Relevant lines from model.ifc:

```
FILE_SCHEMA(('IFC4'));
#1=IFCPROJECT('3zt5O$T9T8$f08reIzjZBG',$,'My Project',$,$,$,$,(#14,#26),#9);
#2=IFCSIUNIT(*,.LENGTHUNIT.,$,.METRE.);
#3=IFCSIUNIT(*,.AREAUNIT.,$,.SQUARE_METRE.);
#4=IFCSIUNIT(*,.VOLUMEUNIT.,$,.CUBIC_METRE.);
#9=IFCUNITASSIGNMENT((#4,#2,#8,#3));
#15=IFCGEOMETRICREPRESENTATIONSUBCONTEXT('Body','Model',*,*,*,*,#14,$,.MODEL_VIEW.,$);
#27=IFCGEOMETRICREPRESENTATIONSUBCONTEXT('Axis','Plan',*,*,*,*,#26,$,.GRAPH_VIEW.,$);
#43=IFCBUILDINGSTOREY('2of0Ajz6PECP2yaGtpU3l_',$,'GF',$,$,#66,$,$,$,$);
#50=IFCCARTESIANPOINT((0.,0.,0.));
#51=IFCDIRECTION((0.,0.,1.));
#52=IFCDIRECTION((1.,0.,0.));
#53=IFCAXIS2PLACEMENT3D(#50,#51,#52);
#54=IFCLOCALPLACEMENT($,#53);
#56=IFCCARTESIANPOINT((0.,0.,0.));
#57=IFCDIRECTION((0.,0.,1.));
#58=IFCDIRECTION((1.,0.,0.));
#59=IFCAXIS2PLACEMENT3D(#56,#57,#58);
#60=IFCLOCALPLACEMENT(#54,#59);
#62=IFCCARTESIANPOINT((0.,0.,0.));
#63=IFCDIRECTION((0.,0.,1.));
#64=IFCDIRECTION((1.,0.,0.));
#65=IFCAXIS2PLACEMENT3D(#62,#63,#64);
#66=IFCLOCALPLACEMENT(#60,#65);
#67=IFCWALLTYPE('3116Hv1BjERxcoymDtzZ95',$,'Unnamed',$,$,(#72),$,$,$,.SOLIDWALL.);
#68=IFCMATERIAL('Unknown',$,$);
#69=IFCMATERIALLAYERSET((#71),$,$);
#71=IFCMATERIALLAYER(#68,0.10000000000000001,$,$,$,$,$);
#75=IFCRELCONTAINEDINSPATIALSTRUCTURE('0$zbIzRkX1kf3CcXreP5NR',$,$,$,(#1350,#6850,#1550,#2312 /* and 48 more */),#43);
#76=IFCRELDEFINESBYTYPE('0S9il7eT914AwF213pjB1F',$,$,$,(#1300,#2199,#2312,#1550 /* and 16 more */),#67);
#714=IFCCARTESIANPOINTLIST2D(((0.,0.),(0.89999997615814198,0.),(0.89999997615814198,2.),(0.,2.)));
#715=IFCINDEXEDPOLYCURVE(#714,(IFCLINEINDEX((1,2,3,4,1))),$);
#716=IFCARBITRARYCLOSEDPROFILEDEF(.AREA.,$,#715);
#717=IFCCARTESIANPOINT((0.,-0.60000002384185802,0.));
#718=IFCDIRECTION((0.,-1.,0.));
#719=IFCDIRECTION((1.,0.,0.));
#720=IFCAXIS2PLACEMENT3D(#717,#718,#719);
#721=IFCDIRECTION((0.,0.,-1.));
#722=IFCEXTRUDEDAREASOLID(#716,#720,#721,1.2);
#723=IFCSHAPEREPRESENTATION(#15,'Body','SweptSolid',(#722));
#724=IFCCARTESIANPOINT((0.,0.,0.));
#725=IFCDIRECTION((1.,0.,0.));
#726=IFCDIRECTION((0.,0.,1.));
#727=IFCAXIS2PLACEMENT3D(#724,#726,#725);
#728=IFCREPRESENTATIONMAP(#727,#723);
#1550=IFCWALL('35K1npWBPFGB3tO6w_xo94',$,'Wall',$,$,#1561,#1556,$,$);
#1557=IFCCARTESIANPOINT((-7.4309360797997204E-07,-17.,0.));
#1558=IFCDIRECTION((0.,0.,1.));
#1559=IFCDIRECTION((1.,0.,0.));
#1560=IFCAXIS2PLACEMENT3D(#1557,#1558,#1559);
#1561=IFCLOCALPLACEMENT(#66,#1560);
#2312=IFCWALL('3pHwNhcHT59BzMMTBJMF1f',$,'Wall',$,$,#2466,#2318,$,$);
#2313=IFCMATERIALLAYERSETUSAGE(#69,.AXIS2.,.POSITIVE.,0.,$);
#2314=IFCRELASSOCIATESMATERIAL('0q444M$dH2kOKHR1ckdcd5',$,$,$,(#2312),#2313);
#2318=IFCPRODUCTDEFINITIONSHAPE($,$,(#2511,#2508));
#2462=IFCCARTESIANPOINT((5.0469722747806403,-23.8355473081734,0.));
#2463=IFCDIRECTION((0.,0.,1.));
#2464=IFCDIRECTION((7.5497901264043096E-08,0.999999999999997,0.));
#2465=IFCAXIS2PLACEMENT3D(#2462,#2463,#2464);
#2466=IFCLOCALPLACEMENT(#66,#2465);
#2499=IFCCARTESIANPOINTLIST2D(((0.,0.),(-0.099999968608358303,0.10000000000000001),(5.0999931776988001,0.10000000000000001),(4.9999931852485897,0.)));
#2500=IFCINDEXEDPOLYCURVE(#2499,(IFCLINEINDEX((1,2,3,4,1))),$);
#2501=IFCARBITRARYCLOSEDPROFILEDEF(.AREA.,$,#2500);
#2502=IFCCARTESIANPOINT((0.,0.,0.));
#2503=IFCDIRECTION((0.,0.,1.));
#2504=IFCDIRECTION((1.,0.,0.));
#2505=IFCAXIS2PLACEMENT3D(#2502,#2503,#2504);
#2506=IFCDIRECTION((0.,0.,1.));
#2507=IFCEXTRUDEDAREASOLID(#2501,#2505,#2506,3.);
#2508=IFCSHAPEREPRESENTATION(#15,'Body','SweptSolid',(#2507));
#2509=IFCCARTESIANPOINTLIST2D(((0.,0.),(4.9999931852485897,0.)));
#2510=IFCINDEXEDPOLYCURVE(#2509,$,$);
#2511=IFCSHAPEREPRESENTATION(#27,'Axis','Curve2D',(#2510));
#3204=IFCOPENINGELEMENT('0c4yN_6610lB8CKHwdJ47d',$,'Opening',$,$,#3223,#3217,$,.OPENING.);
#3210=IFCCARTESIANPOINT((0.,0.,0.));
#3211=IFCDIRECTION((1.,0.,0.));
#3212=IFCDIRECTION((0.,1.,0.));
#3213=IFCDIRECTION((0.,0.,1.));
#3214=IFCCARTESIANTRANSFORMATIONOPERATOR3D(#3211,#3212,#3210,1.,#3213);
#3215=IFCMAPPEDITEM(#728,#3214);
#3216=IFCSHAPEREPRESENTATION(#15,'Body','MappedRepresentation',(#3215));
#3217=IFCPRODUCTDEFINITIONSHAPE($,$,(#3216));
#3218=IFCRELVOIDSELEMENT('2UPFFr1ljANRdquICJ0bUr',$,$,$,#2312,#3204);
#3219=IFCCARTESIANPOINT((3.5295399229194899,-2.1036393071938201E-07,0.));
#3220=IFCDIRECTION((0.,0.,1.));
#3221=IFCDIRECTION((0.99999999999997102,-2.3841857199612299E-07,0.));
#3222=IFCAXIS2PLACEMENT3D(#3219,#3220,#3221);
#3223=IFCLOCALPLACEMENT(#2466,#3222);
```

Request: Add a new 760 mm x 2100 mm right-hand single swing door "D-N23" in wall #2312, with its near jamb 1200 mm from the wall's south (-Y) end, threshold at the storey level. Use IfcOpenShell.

```python
import numpy as np
import ifcopenshell
import ifcopenshell.api.feature
import ifcopenshell.api.geometry
import ifcopenshell.api.root
import ifcopenshell.api.spatial
import ifcopenshell.geom
import ifcopenshell.util.element
import ifcopenshell.util.placement
import ifcopenshell.util.representation
import ifcopenshell.util.shape
import ifcopenshell.util.unit

model = ifcopenshell.open("model.ifc")
unit_scale = ifcopenshell.util.unit.calculate_unit_scale(model)
settings = ifcopenshell.geom.settings()


def volume(element):
    """Net volume in cubic metres, openings subtracted."""
    shape = ifcopenshell.geom.create_shape(settings, element)
    return ifcopenshell.util.shape.get_volume(shape.geometry)


wall = model.by_guid("3pHwNhcHT59BzMMTBJMF1f")
storey = ifcopenshell.util.element.get_container(wall, ifc_class="IfcBuildingStorey")
context = ifcopenshell.util.representation.get_context(model, "Model", "Body", "MODEL_VIEW")
before = volume(wall)

width, height, from_end, sill = 0.76, 2.1, 1.2, 0.0  # metres

# The wall runs along its own X axis, and the end named is its -X end.
wall_shape = ifcopenshell.geom.create_shape(settings, wall)
x, y, z = ifcopenshell.util.shape.get_vertices(wall_shape.geometry).T
start = x.min() + from_end
face, thickness = float(y.min()), float(y.max() - y.min())
wall_matrix = ifcopenshell.util.placement.get_local_placement(wall.ObjectPlacement)
level = ifcopenshell.util.placement.get_local_placement(storey.ObjectPlacement)[2, 3]


def in_wall(x, y):
    """Placement at x, y metres in the wall's axes, at sill height."""
    matrix = wall_matrix.copy()
    matrix[:, 3] = wall_matrix @ np.array([x / unit_scale, y / unit_scale, 0.0, 1.0])
    matrix[2, 3] = level + sill / unit_scale
    return matrix


# Opening: a box that overshoots both wall faces by 50 mm.
opening = ifcopenshell.api.root.create_entity(model, ifc_class="IfcOpeningElement", predefined_type="OPENING")
box = ifcopenshell.api.geometry.add_wall_representation(
    model, context=context, length=width, height=height, thickness=thickness + 0.1
)
ifcopenshell.api.geometry.assign_representation(model, product=opening, representation=box)
ifcopenshell.api.geometry.edit_object_placement(model, product=opening, matrix=in_wall(start, face - 0.05), is_si=False)
ifcopenshell.api.feature.add_feature(model, feature=opening, element=wall)

door = ifcopenshell.api.root.create_entity(model, ifc_class="IfcDoor", name="D-N23", predefined_type="DOOR")
door.OverallWidth, door.OverallHeight = width / unit_scale, height / unit_scale
door.OperationType = "SINGLE_SWING_RIGHT"
body = ifcopenshell.api.geometry.add_door_representation(
    model,
    context=context,
    overall_width=door.OverallWidth,
    overall_height=door.OverallHeight,
    operation_type="SINGLE_SWING_RIGHT",
    lining_properties={"LiningDepth": thickness / unit_scale, "ThresholdDepth": thickness / unit_scale},
)
ifcopenshell.api.geometry.assign_representation(model, product=door, representation=body)
ifcopenshell.api.spatial.assign_container(model, products=[door], relating_structure=storey)
ifcopenshell.api.feature.add_filling(model, opening=opening, element=door)

# The lining spans the wall, so the door starts at the wall face.
ifcopenshell.api.geometry.edit_object_placement(model, product=door, matrix=in_wall(start, face), is_si=False)

after = volume(wall)

print(f"wall volume {before:.3f} -> {after:.3f} m3")

model.write("model_v2.ifc")
```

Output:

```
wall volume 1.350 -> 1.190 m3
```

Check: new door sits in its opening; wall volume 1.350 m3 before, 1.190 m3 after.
